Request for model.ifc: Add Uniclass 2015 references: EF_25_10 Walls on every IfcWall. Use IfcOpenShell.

First a look at what the model holds.

```python
import ifcopenshell

model = ifcopenshell.open("model.ifc")
print(model.schema)
print("classifications:", [c.Name for c in model.by_type("IfcClassification")])
for ifc_class in ("IfcDoor", "IfcRoof", "IfcStair", "IfcWall", "IfcWindow"):
    print(ifc_class, len(model.by_type(ifc_class)))
```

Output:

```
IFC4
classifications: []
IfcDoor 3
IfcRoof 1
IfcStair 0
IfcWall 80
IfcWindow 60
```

```python
import ifcopenshell
import ifcopenshell.api.classification

model = ifcopenshell.open("model.ifc")

system = ifcopenshell.api.classification.add_classification(model, classification="Uniclass 2015")

codes = {
    "IfcWall": ("EF_25_10", "Walls"),
}
for ifc_class, (code, name) in codes.items():
    products = model.by_type(ifc_class)
    ifcopenshell.api.classification.add_reference(
        model, products=products, classification=system, identification=code, name=name
    )
    print(code, len(products))

model.write("model-out.ifc")
```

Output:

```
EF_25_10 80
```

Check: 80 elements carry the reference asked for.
